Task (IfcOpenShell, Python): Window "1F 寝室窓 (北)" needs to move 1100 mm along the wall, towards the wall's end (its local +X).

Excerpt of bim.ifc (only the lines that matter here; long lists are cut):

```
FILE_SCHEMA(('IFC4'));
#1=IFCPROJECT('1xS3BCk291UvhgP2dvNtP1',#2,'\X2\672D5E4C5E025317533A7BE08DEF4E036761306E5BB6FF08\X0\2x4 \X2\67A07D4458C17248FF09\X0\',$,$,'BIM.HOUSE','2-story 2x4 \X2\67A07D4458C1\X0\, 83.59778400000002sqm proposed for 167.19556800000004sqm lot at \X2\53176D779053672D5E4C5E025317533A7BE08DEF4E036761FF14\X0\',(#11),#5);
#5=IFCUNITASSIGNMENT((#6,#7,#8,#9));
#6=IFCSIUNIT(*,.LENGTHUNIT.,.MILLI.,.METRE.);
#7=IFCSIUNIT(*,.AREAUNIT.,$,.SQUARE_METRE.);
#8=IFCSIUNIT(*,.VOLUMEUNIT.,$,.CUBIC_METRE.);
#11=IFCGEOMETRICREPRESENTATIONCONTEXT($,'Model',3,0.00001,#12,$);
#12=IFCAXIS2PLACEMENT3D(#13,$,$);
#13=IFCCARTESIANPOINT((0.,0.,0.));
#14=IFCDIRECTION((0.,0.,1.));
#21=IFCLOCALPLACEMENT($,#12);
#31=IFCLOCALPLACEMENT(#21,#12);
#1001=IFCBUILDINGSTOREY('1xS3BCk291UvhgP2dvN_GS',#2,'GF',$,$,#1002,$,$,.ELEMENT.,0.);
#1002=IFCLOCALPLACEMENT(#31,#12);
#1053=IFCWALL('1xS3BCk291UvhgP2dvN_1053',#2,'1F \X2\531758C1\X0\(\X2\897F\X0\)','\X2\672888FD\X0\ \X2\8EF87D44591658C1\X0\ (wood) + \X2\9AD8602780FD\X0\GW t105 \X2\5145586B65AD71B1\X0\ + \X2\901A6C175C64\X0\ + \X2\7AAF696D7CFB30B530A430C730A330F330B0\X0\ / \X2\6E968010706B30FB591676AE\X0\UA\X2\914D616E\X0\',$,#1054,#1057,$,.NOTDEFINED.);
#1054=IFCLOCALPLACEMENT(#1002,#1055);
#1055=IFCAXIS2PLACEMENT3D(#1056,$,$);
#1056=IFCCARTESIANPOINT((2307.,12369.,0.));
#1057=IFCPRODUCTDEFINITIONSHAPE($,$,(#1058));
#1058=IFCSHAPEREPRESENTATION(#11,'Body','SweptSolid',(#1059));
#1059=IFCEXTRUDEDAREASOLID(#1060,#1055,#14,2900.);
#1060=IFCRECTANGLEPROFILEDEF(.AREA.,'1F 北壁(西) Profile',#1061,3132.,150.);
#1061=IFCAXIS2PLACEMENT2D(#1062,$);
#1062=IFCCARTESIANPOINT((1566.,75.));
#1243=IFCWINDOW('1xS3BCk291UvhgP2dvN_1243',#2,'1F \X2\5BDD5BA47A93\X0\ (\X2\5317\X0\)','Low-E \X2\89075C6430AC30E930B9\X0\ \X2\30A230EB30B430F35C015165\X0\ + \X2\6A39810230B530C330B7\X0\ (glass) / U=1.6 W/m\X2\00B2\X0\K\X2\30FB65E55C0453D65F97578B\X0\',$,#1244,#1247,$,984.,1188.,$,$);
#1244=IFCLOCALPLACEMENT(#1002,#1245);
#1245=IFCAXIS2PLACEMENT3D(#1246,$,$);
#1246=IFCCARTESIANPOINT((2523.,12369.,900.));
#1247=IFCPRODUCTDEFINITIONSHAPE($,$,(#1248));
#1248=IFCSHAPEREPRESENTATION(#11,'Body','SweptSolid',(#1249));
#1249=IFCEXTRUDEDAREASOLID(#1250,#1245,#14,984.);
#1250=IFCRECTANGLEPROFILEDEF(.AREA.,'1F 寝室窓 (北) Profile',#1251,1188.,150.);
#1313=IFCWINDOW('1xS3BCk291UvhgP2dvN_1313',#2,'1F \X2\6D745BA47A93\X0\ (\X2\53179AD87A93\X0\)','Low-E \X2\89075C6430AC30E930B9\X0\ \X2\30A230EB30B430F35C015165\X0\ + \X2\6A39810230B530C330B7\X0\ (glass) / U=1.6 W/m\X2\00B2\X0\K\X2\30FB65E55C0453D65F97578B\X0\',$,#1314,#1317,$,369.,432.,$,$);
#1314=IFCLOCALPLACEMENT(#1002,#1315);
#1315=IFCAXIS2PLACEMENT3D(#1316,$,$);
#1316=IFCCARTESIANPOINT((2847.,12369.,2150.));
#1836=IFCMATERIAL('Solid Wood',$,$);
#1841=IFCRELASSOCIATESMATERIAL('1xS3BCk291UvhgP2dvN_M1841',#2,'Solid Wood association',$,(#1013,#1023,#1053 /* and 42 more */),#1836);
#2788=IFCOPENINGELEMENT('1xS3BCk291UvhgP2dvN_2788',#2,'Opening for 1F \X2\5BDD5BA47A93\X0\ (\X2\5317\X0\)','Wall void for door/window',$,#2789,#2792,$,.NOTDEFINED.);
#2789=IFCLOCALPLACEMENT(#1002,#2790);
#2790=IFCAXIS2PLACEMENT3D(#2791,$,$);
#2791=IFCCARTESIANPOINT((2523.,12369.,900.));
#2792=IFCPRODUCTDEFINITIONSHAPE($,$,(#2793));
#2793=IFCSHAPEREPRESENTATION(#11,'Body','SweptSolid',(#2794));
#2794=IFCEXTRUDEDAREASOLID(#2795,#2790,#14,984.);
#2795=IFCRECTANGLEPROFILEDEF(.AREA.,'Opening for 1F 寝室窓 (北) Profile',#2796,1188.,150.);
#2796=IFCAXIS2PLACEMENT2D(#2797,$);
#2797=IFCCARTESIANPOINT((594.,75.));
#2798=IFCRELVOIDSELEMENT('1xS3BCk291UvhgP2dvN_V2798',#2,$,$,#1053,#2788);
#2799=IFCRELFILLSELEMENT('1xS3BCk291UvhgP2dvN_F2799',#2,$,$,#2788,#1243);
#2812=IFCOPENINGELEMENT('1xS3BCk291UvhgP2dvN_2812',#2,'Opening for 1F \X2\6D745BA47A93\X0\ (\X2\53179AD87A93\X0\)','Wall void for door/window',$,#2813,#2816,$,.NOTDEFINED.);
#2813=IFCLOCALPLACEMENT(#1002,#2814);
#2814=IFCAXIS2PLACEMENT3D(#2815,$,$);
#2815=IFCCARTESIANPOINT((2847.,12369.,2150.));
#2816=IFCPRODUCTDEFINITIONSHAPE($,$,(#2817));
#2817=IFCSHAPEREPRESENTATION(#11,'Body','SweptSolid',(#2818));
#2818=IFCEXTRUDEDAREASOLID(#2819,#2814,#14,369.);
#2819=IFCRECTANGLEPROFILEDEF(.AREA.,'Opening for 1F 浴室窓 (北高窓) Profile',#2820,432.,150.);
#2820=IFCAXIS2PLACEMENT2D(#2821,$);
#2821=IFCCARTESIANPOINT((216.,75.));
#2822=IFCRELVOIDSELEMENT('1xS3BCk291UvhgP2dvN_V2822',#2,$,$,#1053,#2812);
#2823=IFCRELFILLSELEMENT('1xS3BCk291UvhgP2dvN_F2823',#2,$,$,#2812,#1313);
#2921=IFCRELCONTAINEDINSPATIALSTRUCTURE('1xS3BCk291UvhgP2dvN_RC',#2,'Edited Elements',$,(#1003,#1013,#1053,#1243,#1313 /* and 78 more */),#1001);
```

```python
import ifcopenshell
import ifcopenshell.api.geometry
import ifcopenshell.util.placement
import ifcopenshell.util.unit

model = ifcopenshell.open("bim.ifc")
unit_scale = ifcopenshell.util.unit.calculate_unit_scale(model)

window = model.by_id(1243)
opening = window.FillsVoids[0].RelatingOpeningElement
wall = opening.VoidsElements[0].RelatingBuildingElement

wall_matrix = ifcopenshell.util.placement.get_local_placement(wall.ObjectPlacement)
shift = wall_matrix[:3, 0] * 1.1 / unit_scale
before = ifcopenshell.util.placement.get_local_placement(window.ObjectPlacement)[:3, 3].copy()

# The window is not placed relative to its opening, so move both.
for product in (opening, window):
    matrix = ifcopenshell.util.placement.get_local_placement(product.ObjectPlacement)
    matrix[:3, 3] += shift
    ifcopenshell.api.geometry.edit_object_placement(model, product=product, matrix=matrix, is_si=False)

after = ifcopenshell.util.placement.get_local_placement(window.ObjectPlacement)[:3, 3]
print("window moved by", (after - before).round(3) + 0.0)

model.write("bim_edited.ifc")
```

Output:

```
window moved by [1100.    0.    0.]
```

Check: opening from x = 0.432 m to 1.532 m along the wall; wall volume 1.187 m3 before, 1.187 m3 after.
